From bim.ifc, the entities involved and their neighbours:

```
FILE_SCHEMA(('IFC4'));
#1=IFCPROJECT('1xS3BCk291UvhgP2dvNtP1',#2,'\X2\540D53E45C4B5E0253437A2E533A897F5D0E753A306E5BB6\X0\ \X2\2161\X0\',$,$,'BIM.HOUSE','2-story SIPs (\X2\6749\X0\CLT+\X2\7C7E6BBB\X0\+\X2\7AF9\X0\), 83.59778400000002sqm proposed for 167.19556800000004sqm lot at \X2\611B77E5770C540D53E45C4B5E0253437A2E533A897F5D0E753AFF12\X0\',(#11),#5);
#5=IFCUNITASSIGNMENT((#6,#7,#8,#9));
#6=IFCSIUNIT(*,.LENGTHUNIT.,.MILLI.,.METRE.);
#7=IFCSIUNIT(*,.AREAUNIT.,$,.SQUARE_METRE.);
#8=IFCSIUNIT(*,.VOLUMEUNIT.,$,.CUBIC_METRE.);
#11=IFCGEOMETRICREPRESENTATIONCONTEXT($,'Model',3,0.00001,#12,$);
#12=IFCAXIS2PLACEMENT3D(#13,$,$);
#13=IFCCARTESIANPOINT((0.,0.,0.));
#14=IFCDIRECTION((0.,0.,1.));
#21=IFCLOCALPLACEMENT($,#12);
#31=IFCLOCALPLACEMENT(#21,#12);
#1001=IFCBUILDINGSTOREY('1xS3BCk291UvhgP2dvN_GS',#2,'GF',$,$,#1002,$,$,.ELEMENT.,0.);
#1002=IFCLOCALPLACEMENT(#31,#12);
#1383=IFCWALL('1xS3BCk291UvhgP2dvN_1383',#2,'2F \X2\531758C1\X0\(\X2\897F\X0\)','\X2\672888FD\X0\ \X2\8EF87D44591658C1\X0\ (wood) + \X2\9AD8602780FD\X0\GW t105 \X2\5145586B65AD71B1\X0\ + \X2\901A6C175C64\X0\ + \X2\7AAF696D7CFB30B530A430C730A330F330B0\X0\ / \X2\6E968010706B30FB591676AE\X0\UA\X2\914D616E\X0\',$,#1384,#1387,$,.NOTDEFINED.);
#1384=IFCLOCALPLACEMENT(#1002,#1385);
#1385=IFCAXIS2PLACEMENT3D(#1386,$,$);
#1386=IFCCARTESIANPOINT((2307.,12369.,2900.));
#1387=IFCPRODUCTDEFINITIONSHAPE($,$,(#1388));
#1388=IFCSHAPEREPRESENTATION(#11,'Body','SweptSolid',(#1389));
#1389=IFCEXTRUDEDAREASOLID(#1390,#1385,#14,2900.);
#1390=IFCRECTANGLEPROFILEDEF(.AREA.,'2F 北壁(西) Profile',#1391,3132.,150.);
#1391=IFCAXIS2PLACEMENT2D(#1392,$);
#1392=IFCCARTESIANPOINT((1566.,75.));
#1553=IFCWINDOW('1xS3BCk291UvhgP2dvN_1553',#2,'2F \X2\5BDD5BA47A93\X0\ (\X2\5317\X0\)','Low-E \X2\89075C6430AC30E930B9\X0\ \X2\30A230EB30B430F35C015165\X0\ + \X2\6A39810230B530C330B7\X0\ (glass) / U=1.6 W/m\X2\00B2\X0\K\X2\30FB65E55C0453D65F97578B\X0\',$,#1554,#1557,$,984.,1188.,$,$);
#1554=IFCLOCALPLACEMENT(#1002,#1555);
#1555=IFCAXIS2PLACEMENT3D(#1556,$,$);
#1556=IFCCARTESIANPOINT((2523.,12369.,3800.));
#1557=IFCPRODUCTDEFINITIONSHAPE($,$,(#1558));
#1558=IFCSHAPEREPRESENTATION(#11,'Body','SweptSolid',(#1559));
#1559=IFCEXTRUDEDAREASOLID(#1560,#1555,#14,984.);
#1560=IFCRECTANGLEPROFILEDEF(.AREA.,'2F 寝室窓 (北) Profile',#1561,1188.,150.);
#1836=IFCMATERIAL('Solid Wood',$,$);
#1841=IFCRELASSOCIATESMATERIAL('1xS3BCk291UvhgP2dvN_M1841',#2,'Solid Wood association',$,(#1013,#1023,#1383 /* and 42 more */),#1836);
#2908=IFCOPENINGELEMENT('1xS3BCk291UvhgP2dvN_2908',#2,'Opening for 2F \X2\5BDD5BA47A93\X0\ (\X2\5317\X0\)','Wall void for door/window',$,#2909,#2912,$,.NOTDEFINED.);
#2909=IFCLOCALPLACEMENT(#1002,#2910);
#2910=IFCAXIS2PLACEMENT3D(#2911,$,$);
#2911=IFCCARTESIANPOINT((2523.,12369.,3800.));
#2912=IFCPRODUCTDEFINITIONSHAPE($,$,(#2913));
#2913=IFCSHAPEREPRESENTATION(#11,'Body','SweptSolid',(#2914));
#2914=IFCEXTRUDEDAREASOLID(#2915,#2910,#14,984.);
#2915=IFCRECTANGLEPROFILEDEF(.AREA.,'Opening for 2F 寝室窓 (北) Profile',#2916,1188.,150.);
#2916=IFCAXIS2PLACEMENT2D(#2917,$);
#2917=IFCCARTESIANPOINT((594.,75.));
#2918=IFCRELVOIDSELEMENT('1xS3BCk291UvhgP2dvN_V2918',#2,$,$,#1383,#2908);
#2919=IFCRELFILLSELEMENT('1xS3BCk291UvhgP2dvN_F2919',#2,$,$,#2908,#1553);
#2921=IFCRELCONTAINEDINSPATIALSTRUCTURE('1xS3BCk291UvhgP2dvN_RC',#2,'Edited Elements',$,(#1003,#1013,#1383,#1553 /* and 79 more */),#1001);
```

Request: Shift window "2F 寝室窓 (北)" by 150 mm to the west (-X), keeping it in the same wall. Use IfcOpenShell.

```python
import ifcopenshell
import ifcopenshell.api.geometry
import ifcopenshell.util.placement
import ifcopenshell.util.unit

model = ifcopenshell.open("bim.ifc")
unit_scale = ifcopenshell.util.unit.calculate_unit_scale(model)

window = model.by_id(1553)
opening = window.FillsVoids[0].RelatingOpeningElement
wall = opening.VoidsElements[0].RelatingBuildingElement

wall_matrix = ifcopenshell.util.placement.get_local_placement(wall.ObjectPlacement)
shift = wall_matrix[:3, 0] * -0.15 / unit_scale
before = ifcopenshell.util.placement.get_local_placement(window.ObjectPlacement)[:3, 3].copy()

# The window is not placed relative to its opening, so move both.
for product in (opening, window):
    matrix = ifcopenshell.util.placement.get_local_placement(product.ObjectPlacement)
    matrix[:3, 3] += shift
    ifcopenshell.api.geometry.edit_object_placement(model, product=product, matrix=matrix, is_si=False)

after = ifcopenshell.util.placement.get_local_placement(window.ObjectPlacement)[:3, 3]
print("window moved by", (after - before).round(3) + 0.0)

model.write("bim_rev.ifc")
```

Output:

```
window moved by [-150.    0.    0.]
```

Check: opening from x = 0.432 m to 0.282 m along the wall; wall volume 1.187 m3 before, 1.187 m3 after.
